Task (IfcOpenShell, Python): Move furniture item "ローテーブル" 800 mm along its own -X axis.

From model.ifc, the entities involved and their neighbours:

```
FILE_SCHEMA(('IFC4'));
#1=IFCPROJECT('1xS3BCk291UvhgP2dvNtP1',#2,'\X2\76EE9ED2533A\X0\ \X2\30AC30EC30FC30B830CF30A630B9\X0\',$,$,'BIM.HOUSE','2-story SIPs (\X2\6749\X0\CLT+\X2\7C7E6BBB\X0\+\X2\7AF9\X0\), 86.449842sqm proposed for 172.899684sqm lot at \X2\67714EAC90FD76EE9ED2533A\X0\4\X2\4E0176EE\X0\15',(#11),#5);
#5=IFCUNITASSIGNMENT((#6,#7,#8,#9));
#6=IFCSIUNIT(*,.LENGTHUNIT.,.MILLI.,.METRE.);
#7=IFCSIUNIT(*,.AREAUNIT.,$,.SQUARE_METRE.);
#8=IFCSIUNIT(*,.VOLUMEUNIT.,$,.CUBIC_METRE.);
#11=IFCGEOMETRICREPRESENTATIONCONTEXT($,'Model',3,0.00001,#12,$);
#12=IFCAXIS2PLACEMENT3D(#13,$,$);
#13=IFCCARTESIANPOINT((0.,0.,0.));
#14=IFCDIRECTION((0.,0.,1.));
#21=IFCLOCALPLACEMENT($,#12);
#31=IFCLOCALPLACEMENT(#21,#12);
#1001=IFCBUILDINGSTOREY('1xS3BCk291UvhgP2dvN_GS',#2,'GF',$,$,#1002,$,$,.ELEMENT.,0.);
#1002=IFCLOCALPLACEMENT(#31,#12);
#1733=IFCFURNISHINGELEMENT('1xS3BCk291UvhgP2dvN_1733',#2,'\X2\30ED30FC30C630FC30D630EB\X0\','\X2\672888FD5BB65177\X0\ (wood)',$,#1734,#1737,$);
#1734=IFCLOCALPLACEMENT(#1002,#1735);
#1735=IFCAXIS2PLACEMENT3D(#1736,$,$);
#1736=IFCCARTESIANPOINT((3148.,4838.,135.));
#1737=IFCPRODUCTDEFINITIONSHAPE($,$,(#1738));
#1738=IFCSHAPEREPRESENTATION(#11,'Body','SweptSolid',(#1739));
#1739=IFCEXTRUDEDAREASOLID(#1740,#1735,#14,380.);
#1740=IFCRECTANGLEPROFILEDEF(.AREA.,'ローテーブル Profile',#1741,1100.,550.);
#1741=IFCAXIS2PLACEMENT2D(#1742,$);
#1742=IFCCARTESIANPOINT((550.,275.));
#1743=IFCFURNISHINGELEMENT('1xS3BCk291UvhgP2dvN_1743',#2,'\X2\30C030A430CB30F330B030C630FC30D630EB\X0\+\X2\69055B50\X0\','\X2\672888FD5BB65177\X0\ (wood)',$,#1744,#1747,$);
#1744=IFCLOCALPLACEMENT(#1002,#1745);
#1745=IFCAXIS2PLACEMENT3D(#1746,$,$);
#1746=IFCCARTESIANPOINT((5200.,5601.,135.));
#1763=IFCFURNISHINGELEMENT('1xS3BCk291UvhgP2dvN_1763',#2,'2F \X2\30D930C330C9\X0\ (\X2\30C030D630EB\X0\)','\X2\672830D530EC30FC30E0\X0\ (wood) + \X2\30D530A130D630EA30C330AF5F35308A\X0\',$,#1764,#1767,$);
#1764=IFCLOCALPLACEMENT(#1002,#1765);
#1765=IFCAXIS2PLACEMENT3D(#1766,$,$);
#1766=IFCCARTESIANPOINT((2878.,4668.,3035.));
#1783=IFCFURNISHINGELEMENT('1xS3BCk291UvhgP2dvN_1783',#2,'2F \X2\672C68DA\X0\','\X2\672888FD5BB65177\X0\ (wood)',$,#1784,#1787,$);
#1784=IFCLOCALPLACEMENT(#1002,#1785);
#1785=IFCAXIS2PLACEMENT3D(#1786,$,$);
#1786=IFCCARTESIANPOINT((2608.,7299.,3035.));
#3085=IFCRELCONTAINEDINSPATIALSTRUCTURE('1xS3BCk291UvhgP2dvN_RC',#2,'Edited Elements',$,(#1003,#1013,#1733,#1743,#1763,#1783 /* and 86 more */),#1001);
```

```python
import ifcopenshell
import ifcopenshell.api.geometry
import ifcopenshell.util.placement
import ifcopenshell.util.unit

model = ifcopenshell.open("model.ifc")
unit_scale = ifcopenshell.util.unit.calculate_unit_scale(model)

item = model.by_guid("1xS3BCk291UvhgP2dvN_1733")
matrix = ifcopenshell.util.placement.get_local_placement(item.ObjectPlacement)
matrix[:3, 3] -= matrix[:3, 0] * 0.8 / unit_scale
ifcopenshell.api.geometry.edit_object_placement(model, product=item, matrix=matrix, is_si=False)

print(ifcopenshell.util.placement.get_local_placement(item.ObjectPlacement).round(3) + 0.0)

model.write("model_v2.ifc")
```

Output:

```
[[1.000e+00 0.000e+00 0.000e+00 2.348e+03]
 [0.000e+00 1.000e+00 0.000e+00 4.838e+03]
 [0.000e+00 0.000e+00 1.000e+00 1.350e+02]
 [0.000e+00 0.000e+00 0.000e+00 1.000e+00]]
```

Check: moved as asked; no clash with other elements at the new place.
